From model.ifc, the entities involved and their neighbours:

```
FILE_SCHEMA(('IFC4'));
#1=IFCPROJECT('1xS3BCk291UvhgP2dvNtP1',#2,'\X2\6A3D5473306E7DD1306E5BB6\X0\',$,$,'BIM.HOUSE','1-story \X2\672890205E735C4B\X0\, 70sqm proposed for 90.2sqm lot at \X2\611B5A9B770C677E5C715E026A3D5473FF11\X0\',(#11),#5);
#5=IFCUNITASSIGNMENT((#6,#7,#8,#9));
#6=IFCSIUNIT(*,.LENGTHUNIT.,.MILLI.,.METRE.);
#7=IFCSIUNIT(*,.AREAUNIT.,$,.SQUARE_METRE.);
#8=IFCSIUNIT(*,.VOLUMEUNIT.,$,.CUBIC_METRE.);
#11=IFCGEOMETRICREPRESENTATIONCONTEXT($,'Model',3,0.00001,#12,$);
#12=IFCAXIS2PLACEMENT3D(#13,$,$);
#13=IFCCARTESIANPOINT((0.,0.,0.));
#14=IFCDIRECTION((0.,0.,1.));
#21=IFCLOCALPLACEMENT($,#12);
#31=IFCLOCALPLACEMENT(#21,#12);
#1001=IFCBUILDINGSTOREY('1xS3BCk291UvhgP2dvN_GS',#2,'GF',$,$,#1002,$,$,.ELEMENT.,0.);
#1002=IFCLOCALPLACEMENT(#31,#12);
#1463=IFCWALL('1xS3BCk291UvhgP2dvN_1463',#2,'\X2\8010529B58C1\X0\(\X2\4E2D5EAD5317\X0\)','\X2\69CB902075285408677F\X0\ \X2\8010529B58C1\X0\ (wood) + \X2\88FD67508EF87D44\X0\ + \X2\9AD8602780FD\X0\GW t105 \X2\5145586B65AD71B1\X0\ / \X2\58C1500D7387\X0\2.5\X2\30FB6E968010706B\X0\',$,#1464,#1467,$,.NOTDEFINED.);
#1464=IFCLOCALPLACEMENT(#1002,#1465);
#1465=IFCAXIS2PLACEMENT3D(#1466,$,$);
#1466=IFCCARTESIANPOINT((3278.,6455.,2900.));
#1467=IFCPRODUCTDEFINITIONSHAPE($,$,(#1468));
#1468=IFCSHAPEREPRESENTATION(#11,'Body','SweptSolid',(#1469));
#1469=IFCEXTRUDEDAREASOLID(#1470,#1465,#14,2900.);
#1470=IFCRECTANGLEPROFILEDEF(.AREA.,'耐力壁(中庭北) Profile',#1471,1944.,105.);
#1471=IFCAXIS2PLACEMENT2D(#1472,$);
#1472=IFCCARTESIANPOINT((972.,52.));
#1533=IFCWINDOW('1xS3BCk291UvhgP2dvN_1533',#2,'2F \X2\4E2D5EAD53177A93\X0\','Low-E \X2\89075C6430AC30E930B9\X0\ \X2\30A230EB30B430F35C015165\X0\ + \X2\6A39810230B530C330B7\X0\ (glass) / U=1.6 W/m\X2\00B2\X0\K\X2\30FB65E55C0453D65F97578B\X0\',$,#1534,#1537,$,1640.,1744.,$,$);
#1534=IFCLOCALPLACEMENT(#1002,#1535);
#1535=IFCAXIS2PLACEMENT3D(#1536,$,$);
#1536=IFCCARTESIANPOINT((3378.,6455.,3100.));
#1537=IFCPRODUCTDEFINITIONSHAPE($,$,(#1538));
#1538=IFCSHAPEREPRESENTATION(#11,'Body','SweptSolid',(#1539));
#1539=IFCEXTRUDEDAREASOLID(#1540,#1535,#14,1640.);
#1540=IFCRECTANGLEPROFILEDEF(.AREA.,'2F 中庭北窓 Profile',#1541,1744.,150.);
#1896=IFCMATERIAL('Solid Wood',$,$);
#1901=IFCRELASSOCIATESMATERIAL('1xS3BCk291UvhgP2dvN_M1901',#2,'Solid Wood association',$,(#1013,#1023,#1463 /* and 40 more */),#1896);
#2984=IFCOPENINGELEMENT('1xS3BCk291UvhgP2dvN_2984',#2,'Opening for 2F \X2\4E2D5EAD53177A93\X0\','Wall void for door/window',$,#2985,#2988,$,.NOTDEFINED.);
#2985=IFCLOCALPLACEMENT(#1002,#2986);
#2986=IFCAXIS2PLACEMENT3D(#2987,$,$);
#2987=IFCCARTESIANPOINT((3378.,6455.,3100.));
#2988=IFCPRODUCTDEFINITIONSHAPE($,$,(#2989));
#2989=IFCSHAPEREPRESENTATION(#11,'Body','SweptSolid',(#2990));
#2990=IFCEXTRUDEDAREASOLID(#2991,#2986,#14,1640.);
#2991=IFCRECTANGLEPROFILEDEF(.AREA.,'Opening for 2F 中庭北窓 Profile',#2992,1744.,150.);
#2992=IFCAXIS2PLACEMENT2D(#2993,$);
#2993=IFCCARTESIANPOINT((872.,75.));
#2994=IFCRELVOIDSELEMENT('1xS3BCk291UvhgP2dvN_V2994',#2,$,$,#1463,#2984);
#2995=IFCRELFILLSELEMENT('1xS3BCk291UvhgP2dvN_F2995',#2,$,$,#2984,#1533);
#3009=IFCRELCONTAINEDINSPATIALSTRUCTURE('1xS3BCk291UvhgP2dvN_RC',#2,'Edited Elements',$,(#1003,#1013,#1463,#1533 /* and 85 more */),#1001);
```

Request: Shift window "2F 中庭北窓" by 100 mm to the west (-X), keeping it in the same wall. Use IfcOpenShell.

```python
import ifcopenshell
import ifcopenshell.api.geometry
import ifcopenshell.util.placement
import ifcopenshell.util.unit

model = ifcopenshell.open("model.ifc")
unit_scale = ifcopenshell.util.unit.calculate_unit_scale(model)

window = model.by_id(1533)
opening = window.FillsVoids[0].RelatingOpeningElement
wall = opening.VoidsElements[0].RelatingBuildingElement

wall_matrix = ifcopenshell.util.placement.get_local_placement(wall.ObjectPlacement)
shift = wall_matrix[:3, 0] * -0.1 / unit_scale
before = ifcopenshell.util.placement.get_local_placement(window.ObjectPlacement)[:3, 3].copy()

# The window is not placed relative to its opening, so move both.
for product in (opening, window):
    matrix = ifcopenshell.util.placement.get_local_placement(product.ObjectPlacement)
    matrix[:3, 3] += shift
    ifcopenshell.api.geometry.edit_object_placement(model, product=product, matrix=matrix, is_si=False)

after = ifcopenshell.util.placement.get_local_placement(window.ObjectPlacement)[:3, 3]
print("window moved by", (after - before).round(3) + 0.0)

model.write("model_updated.ifc")
```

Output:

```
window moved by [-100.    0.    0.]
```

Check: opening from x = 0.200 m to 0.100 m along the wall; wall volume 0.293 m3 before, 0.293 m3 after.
